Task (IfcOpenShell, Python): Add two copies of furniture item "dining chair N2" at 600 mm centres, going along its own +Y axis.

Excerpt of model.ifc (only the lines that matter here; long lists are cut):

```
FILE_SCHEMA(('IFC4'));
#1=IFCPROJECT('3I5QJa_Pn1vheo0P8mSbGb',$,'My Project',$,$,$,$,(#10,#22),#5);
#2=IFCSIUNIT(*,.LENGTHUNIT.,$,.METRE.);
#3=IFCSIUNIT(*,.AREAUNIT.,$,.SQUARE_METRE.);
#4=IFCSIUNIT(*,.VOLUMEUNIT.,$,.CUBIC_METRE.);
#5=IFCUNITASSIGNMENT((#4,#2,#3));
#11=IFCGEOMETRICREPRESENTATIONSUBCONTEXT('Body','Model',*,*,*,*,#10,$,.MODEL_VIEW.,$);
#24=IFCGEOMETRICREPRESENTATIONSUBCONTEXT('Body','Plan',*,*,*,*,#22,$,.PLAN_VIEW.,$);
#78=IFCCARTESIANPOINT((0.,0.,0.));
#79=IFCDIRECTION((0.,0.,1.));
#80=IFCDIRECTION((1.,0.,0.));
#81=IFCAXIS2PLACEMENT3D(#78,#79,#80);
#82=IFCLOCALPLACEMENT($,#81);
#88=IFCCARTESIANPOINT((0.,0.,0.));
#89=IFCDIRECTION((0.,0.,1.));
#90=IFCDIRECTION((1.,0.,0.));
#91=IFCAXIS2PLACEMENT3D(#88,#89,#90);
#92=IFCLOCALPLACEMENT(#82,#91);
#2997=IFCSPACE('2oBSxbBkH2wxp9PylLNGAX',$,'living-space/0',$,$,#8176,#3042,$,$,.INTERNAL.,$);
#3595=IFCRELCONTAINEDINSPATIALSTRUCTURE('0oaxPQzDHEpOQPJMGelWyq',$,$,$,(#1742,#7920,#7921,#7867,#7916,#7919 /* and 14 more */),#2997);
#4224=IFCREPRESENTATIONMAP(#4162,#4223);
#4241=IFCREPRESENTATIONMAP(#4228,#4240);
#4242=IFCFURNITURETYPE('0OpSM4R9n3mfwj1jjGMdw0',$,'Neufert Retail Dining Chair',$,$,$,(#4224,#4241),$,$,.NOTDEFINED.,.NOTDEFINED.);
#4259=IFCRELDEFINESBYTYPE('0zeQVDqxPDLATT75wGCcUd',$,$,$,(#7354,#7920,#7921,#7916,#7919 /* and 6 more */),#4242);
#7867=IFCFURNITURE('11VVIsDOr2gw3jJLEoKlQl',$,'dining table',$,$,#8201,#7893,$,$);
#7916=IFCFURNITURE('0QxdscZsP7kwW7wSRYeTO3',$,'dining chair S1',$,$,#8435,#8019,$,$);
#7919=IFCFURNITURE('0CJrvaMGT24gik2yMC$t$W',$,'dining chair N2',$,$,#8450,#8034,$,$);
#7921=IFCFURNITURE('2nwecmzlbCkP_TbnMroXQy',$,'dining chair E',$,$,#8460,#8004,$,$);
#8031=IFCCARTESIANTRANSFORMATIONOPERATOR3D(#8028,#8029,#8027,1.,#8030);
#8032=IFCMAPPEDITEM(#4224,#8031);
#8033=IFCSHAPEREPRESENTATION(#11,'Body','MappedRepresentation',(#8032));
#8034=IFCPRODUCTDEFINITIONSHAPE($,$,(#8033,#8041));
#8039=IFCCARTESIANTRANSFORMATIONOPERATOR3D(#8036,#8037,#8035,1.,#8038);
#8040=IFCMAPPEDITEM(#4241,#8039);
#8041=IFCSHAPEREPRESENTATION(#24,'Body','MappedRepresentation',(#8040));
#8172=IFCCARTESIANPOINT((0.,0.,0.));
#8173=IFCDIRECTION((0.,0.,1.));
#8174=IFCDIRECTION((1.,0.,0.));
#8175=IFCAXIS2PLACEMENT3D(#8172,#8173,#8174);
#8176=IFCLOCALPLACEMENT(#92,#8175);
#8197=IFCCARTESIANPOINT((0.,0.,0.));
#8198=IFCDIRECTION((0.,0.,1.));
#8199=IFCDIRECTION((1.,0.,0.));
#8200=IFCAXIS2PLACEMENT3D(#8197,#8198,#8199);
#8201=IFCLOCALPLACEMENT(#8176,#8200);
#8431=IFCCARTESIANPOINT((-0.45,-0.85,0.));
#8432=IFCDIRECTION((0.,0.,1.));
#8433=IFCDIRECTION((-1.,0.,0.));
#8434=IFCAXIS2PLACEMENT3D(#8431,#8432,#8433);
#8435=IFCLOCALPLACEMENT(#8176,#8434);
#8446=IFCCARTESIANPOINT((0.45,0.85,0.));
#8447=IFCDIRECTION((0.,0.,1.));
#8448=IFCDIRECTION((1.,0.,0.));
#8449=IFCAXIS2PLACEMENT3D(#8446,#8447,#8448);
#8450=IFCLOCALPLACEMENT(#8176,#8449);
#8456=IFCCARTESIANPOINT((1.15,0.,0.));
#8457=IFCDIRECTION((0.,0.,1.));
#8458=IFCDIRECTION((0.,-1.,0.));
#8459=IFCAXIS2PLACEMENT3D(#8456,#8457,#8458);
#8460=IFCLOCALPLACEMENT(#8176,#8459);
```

```python
import ifcopenshell
import ifcopenshell.api.geometry
import ifcopenshell.api.root
import ifcopenshell.util.element
import ifcopenshell.util.placement
import ifcopenshell.util.unit

model = ifcopenshell.open("model.ifc")
unit_scale = ifcopenshell.util.unit.calculate_unit_scale(model)

source = model.by_guid("0CJrvaMGT24gik2yMC$t$W")
base = ifcopenshell.util.placement.get_local_placement(source.ObjectPlacement)
step = base[:3, 1] * 0.6 / unit_scale

for i in range(1, 3):
    copy = ifcopenshell.api.root.copy_class(model, product=source)
    copy.Representation = ifcopenshell.util.element.copy_deep(
        model, source.Representation, exclude=["IfcGeometricRepresentationContext", "IfcRepresentationMap"]
    )
    matrix = base.copy()
    matrix[:3, 3] += i * step
    print("added at", matrix[:3, 3].round(3) + 0.0)
    ifcopenshell.api.geometry.edit_object_placement(model, product=copy, matrix=matrix, is_si=False)

model.write("model_edited.ifc")
```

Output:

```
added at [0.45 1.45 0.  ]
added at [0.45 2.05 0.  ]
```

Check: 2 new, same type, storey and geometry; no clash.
